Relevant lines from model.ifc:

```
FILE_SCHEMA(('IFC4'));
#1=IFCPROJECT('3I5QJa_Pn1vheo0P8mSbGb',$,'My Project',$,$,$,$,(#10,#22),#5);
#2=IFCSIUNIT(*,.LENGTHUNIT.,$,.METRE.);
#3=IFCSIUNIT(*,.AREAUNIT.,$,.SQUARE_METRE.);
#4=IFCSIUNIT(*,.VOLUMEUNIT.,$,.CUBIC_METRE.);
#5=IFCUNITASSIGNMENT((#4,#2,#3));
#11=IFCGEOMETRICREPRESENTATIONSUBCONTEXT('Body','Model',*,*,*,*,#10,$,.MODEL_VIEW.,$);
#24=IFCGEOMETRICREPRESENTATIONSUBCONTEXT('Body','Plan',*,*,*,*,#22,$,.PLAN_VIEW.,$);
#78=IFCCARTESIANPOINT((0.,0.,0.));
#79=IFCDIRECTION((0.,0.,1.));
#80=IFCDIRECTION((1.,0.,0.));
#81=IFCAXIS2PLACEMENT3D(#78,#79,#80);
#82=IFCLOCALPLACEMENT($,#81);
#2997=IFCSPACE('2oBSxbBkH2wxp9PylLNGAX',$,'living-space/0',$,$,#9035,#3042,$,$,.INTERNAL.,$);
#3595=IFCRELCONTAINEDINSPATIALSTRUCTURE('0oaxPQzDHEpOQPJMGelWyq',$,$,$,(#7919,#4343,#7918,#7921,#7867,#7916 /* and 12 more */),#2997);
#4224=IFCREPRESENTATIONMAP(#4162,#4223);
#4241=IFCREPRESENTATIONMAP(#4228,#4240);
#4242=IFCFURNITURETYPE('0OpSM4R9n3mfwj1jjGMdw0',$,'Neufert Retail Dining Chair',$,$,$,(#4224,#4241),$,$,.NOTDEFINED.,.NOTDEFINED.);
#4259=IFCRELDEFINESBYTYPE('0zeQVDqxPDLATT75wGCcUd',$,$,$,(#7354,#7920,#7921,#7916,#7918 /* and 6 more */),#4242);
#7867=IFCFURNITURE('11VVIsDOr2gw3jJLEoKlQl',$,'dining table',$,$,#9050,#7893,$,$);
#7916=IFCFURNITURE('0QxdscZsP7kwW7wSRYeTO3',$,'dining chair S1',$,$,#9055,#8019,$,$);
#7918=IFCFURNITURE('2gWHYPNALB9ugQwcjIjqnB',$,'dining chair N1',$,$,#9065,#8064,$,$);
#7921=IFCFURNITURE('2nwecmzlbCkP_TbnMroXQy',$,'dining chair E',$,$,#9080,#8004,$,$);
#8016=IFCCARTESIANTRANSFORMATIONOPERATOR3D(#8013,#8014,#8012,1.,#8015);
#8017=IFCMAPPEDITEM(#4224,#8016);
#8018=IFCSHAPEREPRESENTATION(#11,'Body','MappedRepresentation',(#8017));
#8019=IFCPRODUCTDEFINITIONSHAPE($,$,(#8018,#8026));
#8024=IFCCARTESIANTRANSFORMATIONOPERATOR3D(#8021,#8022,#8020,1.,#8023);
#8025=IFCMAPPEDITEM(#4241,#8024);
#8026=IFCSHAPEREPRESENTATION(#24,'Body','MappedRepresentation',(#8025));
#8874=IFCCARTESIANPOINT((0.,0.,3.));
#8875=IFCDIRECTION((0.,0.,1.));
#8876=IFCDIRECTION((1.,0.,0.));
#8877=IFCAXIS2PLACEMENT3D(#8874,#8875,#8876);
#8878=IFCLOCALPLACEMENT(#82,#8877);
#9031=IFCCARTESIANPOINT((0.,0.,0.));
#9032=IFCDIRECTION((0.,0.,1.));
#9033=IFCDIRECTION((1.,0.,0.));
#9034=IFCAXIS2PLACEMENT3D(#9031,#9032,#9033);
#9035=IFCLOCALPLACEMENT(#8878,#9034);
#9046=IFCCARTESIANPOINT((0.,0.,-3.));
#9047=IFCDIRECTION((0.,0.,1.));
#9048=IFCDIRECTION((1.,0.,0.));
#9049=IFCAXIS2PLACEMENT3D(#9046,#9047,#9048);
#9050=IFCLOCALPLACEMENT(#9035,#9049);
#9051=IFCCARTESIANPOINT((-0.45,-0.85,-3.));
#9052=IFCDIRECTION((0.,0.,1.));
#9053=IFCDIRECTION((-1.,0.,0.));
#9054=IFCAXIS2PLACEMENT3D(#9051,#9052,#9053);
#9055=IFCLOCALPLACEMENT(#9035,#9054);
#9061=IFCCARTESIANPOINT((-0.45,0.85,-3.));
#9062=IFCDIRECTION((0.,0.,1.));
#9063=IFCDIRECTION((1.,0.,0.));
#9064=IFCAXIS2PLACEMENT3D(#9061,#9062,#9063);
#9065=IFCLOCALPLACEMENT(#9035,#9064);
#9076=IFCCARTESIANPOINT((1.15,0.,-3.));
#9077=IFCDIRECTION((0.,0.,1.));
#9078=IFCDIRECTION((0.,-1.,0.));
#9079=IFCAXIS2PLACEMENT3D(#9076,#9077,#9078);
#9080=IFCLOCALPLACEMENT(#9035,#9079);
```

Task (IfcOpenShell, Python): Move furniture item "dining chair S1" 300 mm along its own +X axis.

```python
import ifcopenshell
import ifcopenshell.api.geometry
import ifcopenshell.util.placement

model = ifcopenshell.open("model.ifc")

item = model.by_guid("0QxdscZsP7kwW7wSRYeTO3")
matrix = ifcopenshell.util.placement.get_local_placement(item.ObjectPlacement)
matrix[:3, 3] += matrix[:3, 0] * 0.3
ifcopenshell.api.geometry.edit_object_placement(model, product=item, matrix=matrix, is_si=False)

print(ifcopenshell.util.placement.get_local_placement(item.ObjectPlacement).round(3) + 0.0)

model.write("model_v2.ifc")
```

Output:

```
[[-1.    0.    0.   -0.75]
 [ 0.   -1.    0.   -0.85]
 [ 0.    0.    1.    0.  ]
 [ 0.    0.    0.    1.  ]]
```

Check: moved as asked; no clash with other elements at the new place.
